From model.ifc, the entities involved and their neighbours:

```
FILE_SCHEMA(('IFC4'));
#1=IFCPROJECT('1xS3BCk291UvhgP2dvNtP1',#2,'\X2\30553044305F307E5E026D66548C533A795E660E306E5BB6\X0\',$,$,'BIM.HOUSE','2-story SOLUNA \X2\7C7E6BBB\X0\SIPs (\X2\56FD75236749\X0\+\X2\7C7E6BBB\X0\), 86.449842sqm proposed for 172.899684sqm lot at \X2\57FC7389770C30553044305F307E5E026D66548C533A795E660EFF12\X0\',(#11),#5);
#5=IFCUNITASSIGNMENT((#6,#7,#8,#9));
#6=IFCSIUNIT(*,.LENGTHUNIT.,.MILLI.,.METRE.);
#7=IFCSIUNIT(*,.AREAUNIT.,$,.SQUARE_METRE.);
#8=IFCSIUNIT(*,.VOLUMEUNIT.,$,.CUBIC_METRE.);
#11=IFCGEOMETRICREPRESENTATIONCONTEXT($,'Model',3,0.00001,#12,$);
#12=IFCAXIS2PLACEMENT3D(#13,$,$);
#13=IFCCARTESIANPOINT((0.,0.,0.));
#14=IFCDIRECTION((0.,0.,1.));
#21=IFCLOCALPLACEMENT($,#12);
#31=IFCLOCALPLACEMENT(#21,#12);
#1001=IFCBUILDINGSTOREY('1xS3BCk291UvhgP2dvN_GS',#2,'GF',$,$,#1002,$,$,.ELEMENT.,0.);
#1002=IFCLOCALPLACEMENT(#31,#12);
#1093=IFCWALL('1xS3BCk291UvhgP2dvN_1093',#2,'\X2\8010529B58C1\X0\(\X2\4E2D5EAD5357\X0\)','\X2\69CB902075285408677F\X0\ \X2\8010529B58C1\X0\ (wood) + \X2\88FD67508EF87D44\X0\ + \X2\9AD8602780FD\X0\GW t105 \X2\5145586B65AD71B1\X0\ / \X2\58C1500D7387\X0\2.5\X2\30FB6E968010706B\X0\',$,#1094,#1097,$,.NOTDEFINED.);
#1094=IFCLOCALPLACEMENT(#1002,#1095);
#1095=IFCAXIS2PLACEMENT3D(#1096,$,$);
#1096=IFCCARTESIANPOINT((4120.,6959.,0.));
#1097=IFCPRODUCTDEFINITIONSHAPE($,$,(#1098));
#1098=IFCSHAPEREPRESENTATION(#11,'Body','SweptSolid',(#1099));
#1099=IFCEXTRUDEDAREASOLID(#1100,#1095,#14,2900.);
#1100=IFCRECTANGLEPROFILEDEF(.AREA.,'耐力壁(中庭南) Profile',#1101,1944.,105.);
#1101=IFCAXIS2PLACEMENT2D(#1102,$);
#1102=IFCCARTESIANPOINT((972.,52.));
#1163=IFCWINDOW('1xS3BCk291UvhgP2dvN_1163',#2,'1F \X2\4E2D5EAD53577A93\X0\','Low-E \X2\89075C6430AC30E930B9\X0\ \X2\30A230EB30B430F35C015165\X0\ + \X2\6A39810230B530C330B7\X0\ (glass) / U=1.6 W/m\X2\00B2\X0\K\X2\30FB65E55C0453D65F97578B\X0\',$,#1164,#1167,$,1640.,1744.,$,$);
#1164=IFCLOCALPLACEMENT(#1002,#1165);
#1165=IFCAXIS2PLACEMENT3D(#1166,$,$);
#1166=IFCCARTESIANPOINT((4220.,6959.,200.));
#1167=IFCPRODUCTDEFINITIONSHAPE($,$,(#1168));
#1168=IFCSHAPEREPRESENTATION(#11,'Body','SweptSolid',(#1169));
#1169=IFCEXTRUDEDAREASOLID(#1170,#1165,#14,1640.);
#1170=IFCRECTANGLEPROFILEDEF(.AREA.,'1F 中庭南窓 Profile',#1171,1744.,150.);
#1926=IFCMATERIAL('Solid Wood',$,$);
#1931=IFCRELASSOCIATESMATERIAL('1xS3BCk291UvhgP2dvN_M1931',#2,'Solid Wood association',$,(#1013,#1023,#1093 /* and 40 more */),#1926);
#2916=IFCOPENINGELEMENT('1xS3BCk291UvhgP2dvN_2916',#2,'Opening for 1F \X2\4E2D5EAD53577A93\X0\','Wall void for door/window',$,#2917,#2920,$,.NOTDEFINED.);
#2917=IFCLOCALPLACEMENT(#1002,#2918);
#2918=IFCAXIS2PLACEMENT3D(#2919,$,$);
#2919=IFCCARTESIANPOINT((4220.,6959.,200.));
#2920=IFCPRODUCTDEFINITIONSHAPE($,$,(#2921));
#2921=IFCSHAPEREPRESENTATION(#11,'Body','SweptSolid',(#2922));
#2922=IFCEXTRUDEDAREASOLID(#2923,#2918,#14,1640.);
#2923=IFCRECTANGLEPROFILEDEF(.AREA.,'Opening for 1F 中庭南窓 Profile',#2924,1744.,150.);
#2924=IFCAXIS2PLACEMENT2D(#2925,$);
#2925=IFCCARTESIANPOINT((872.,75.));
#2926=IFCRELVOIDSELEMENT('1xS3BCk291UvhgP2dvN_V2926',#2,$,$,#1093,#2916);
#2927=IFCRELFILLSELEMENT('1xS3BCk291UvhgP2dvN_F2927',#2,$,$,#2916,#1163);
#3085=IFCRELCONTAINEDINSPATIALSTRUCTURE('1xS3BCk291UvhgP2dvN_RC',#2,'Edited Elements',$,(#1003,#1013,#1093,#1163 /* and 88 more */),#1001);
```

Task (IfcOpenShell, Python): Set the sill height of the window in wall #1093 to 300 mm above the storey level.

```python
import numpy as np
import ifcopenshell
import ifcopenshell.api.geometry
import ifcopenshell.geom
import ifcopenshell.util.element
import ifcopenshell.util.placement
import ifcopenshell.util.shape
import ifcopenshell.util.unit

model = ifcopenshell.open("model.ifc")
unit_scale = ifcopenshell.util.unit.calculate_unit_scale(model)

window = model.by_guid("1xS3BCk291UvhgP2dvN_1163")
opening = window.FillsVoids[0].RelatingOpeningElement
storey = ifcopenshell.util.element.get_container(window, ifc_class="IfcBuildingStorey")
level = ifcopenshell.util.placement.get_local_placement(storey.ObjectPlacement)[2, 3]

# The opening's origin need not be at the sill, so measure its lowest point.
shape = ifcopenshell.geom.create_shape(ifcopenshell.geom.settings(), opening)
bottom = ifcopenshell.util.shape.get_shape_bottom_elevation(shape, shape.geometry) / unit_scale
dz = level + 0.3 / unit_scale - bottom

shift = np.array([0.0, 0.0, dz])
# The window is not placed relative to its opening, so move both.
for product in (opening, window):
    matrix = ifcopenshell.util.placement.get_local_placement(product.ObjectPlacement)
    matrix[:3, 3] += shift
    ifcopenshell.api.geometry.edit_object_placement(model, product=product, matrix=matrix, is_si=False)

print(f"moved by {dz * unit_scale:+.3f} m")

model.write("model_rev.ifc")
```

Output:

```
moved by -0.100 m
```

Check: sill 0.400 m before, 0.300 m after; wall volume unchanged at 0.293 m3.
